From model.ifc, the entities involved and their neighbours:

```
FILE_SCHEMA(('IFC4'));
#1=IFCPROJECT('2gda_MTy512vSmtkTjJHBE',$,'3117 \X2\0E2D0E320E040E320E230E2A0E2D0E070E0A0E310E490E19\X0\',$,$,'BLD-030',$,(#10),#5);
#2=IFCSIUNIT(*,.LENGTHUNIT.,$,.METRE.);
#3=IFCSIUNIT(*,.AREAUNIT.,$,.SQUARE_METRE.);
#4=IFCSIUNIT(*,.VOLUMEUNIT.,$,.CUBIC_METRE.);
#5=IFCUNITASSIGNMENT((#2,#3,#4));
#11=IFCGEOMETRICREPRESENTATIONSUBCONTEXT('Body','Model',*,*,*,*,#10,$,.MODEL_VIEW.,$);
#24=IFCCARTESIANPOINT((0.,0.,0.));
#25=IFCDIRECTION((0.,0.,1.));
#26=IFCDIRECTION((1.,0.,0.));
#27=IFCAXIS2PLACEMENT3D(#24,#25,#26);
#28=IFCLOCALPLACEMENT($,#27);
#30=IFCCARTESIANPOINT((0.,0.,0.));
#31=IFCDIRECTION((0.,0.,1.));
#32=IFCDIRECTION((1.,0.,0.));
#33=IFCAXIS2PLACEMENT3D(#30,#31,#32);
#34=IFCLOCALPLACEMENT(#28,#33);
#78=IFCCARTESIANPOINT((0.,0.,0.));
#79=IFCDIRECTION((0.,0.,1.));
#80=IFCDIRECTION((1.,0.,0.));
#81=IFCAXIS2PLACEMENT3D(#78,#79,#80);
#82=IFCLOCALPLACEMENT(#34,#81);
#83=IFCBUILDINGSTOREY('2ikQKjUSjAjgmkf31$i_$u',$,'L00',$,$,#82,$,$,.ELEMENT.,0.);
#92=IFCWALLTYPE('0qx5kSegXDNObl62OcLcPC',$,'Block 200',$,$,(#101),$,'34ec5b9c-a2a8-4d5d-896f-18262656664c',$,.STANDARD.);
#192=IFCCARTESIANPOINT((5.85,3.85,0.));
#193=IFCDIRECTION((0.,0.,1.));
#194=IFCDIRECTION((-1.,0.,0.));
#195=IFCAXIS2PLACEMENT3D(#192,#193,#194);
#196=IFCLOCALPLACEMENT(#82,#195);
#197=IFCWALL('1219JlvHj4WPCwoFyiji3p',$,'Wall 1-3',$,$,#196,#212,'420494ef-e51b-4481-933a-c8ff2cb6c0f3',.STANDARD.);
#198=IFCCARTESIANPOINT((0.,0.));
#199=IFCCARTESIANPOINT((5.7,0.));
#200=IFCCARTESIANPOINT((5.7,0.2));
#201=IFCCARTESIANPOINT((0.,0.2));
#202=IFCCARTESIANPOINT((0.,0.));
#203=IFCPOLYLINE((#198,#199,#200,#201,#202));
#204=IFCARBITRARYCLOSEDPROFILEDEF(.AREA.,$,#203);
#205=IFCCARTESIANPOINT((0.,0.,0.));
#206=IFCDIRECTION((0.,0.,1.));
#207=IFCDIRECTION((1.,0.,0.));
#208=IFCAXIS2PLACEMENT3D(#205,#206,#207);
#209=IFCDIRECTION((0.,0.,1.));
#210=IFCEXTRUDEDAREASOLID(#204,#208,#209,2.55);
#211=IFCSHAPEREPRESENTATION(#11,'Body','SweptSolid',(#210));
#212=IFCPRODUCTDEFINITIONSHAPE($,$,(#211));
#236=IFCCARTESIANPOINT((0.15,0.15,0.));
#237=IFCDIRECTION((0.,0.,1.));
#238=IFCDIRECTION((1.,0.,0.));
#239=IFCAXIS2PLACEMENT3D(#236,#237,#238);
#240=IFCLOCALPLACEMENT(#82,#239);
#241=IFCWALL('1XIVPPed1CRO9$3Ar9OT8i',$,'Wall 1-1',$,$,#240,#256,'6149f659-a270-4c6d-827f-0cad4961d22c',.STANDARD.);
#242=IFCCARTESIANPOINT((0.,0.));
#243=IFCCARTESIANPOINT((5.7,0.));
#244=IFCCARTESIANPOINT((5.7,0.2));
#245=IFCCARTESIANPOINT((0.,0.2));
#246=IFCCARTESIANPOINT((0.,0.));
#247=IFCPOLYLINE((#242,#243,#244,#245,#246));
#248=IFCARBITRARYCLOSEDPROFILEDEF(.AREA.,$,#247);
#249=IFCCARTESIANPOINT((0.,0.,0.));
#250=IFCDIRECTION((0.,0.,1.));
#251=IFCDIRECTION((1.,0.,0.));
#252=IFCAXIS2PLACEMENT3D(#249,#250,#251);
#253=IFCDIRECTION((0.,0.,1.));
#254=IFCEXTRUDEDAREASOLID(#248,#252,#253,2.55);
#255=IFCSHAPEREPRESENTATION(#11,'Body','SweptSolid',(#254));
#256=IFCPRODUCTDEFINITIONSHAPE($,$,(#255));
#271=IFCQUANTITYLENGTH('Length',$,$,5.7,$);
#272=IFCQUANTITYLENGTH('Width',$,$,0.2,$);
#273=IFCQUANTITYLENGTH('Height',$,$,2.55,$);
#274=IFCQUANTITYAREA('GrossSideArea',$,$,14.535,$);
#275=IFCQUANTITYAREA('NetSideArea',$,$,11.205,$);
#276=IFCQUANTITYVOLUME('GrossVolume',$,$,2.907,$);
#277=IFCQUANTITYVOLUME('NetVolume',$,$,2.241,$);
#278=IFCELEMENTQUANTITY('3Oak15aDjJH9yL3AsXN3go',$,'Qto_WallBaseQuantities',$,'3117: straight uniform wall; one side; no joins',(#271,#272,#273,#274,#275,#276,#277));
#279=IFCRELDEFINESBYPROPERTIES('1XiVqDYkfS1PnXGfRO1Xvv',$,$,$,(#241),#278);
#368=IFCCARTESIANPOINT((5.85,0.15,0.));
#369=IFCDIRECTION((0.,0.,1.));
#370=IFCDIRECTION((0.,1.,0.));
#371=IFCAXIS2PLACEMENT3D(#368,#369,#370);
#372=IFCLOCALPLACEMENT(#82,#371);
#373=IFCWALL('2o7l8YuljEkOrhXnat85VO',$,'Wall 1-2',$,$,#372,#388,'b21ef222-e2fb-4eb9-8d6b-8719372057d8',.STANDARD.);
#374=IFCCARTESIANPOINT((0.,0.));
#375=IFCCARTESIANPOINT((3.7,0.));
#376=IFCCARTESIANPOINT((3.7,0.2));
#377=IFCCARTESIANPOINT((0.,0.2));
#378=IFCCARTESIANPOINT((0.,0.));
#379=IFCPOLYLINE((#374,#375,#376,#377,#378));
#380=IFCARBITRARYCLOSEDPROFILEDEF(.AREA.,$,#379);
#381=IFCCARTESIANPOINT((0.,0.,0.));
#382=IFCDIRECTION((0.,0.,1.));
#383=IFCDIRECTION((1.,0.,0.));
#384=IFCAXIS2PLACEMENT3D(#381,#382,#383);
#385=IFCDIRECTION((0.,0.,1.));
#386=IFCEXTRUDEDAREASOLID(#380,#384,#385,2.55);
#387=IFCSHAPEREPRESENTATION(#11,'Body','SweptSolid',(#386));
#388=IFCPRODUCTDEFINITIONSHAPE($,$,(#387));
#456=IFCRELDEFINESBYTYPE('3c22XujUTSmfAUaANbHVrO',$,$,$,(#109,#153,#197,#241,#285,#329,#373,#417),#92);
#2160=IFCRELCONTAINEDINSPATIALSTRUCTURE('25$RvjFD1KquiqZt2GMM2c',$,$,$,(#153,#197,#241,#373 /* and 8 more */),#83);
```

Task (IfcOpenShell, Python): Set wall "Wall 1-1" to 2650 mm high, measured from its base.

```python
import ifcopenshell
import ifcopenshell.api.pset
import ifcopenshell.geom
import ifcopenshell.util.element
import ifcopenshell.util.representation
import ifcopenshell.util.shape
import ifcopenshell.util.unit

model = ifcopenshell.open("model.ifc")
unit_scale = ifcopenshell.util.unit.calculate_unit_scale(model)
area_scale = ifcopenshell.util.unit.calculate_unit_scale(model, "AREAUNIT")
volume_scale = ifcopenshell.util.unit.calculate_unit_scale(model, "VOLUMEUNIT")
settings = ifcopenshell.geom.settings()


def volume(element):
    """Net volume in cubic metres, openings subtracted."""
    shape = ifcopenshell.geom.create_shape(settings, element)
    return ifcopenshell.util.shape.get_volume(shape.geometry)


wall = model.by_guid("1XIVPPed1CRO9$3Ar9OT8i")
before = volume(wall)

body = ifcopenshell.util.representation.get_representation(wall, "Model", "Body")
solid = body.Items[0]
old_height = solid.Depth
solid.Depth = 2.65 / unit_scale
after = volume(wall)
thickness = 0.2  # wall thickness in metres

# Update the stored height, areas and volumes.
qto = model.by_id(ifcopenshell.util.element.get_pset(wall, "Qto_WallBaseQuantities", should_inherit=False)["id"])
ifcopenshell.api.pset.edit_qto(model, qto=qto, properties={
    "Height": solid.Depth,
    "GrossSideArea": ifcopenshell.util.element.get_pset(wall, "Qto_WallBaseQuantities", "GrossSideArea") * solid.Depth / old_height,
    "NetSideArea": after / thickness / area_scale,
    "GrossVolume": ifcopenshell.util.element.get_pset(wall, "Qto_WallBaseQuantities", "GrossVolume") * solid.Depth / old_height,
    "NetVolume": after / volume_scale,
})

print(f"height {old_height:g} -> {solid.Depth:g}, volume {before:.3f} -> {after:.3f} m3")

model.write("model_v2.ifc")
```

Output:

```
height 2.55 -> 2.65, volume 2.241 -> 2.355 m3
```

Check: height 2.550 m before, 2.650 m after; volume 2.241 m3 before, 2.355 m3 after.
